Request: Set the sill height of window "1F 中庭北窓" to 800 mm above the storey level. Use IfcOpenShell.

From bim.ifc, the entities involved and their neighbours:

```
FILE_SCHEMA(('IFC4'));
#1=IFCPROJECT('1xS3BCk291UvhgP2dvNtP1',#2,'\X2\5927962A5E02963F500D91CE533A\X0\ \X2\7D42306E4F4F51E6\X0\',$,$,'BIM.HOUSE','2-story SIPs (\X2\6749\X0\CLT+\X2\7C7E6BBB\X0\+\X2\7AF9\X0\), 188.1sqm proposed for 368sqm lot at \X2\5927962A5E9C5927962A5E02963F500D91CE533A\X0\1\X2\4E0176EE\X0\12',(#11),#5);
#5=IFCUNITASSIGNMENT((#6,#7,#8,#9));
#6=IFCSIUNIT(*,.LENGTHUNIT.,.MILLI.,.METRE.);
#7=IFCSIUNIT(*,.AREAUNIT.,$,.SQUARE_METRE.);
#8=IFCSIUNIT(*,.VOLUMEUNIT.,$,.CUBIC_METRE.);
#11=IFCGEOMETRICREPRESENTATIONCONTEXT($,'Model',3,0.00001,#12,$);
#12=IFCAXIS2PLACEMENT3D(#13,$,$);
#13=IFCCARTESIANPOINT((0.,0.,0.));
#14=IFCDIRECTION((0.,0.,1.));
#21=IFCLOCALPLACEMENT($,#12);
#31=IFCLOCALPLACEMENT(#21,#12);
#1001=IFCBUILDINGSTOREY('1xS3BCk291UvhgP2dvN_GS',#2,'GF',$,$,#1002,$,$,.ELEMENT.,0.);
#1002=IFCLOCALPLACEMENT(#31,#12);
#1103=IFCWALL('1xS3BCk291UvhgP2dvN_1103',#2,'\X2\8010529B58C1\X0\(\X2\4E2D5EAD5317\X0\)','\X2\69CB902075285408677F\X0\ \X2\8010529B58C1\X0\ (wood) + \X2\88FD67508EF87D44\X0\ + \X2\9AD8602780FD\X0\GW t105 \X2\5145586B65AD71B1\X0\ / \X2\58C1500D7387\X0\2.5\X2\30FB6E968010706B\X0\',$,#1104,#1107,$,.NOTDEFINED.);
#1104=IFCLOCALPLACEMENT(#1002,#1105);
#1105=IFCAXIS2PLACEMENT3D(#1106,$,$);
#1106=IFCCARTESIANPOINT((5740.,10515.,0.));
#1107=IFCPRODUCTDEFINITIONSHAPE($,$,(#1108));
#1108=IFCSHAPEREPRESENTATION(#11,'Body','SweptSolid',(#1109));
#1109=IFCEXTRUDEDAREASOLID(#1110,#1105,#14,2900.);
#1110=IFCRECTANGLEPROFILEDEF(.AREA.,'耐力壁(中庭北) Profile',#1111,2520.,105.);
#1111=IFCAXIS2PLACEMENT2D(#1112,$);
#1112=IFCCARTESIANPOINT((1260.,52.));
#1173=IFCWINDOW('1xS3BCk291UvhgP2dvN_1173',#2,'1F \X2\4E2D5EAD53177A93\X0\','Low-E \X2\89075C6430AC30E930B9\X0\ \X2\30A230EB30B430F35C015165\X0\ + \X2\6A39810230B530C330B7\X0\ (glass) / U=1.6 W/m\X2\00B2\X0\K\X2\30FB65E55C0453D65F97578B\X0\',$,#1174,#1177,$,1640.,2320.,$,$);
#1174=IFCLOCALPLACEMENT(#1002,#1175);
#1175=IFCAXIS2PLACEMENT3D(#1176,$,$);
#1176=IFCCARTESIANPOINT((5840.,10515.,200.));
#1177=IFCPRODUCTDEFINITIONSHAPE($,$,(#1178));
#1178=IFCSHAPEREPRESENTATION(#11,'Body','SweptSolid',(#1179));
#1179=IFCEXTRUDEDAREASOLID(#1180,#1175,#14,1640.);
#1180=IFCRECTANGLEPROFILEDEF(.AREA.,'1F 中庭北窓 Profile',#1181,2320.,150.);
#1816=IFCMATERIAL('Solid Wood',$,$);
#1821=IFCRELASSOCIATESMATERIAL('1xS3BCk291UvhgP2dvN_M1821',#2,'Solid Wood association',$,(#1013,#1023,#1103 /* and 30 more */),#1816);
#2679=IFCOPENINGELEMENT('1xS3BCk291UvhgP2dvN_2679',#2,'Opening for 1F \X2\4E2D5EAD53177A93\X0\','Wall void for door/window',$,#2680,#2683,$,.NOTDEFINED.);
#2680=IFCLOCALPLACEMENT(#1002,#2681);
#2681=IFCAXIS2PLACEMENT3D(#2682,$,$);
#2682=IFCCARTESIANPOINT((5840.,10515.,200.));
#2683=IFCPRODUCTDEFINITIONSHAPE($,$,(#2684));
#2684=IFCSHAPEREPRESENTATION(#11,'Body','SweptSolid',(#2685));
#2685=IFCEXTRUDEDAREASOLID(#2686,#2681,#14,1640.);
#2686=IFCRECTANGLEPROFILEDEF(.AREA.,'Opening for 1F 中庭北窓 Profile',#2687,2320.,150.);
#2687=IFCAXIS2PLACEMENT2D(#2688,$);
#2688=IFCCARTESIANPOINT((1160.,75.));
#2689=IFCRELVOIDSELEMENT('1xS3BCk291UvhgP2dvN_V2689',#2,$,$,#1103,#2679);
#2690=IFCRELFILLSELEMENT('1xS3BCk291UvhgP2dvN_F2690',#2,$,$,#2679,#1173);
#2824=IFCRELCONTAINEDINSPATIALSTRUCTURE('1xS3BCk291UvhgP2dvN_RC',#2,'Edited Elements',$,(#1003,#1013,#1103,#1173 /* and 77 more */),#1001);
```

```python
import numpy as np
import ifcopenshell
import ifcopenshell.api.geometry
import ifcopenshell.geom
import ifcopenshell.util.element
import ifcopenshell.util.placement
import ifcopenshell.util.shape
import ifcopenshell.util.unit

model = ifcopenshell.open("bim.ifc")
unit_scale = ifcopenshell.util.unit.calculate_unit_scale(model)

window = model.by_guid("1xS3BCk291UvhgP2dvN_1173")
opening = window.FillsVoids[0].RelatingOpeningElement
storey = ifcopenshell.util.element.get_container(window, ifc_class="IfcBuildingStorey")
level = ifcopenshell.util.placement.get_local_placement(storey.ObjectPlacement)[2, 3]

# The opening's origin need not be at the sill, so measure its lowest point.
shape = ifcopenshell.geom.create_shape(ifcopenshell.geom.settings(), opening)
bottom = ifcopenshell.util.shape.get_shape_bottom_elevation(shape, shape.geometry) / unit_scale
dz = level + 0.8 / unit_scale - bottom

shift = np.array([0.0, 0.0, dz])
# The window is not placed relative to its opening, so move both.
for product in (opening, window):
    matrix = ifcopenshell.util.placement.get_local_placement(product.ObjectPlacement)
    matrix[:3, 3] += shift
    ifcopenshell.api.geometry.edit_object_placement(model, product=product, matrix=matrix, is_si=False)

print(f"moved by {dz * unit_scale:+.3f} m")

model.write("bim_v2.ifc")
```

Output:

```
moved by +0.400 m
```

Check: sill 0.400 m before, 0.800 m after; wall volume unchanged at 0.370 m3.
